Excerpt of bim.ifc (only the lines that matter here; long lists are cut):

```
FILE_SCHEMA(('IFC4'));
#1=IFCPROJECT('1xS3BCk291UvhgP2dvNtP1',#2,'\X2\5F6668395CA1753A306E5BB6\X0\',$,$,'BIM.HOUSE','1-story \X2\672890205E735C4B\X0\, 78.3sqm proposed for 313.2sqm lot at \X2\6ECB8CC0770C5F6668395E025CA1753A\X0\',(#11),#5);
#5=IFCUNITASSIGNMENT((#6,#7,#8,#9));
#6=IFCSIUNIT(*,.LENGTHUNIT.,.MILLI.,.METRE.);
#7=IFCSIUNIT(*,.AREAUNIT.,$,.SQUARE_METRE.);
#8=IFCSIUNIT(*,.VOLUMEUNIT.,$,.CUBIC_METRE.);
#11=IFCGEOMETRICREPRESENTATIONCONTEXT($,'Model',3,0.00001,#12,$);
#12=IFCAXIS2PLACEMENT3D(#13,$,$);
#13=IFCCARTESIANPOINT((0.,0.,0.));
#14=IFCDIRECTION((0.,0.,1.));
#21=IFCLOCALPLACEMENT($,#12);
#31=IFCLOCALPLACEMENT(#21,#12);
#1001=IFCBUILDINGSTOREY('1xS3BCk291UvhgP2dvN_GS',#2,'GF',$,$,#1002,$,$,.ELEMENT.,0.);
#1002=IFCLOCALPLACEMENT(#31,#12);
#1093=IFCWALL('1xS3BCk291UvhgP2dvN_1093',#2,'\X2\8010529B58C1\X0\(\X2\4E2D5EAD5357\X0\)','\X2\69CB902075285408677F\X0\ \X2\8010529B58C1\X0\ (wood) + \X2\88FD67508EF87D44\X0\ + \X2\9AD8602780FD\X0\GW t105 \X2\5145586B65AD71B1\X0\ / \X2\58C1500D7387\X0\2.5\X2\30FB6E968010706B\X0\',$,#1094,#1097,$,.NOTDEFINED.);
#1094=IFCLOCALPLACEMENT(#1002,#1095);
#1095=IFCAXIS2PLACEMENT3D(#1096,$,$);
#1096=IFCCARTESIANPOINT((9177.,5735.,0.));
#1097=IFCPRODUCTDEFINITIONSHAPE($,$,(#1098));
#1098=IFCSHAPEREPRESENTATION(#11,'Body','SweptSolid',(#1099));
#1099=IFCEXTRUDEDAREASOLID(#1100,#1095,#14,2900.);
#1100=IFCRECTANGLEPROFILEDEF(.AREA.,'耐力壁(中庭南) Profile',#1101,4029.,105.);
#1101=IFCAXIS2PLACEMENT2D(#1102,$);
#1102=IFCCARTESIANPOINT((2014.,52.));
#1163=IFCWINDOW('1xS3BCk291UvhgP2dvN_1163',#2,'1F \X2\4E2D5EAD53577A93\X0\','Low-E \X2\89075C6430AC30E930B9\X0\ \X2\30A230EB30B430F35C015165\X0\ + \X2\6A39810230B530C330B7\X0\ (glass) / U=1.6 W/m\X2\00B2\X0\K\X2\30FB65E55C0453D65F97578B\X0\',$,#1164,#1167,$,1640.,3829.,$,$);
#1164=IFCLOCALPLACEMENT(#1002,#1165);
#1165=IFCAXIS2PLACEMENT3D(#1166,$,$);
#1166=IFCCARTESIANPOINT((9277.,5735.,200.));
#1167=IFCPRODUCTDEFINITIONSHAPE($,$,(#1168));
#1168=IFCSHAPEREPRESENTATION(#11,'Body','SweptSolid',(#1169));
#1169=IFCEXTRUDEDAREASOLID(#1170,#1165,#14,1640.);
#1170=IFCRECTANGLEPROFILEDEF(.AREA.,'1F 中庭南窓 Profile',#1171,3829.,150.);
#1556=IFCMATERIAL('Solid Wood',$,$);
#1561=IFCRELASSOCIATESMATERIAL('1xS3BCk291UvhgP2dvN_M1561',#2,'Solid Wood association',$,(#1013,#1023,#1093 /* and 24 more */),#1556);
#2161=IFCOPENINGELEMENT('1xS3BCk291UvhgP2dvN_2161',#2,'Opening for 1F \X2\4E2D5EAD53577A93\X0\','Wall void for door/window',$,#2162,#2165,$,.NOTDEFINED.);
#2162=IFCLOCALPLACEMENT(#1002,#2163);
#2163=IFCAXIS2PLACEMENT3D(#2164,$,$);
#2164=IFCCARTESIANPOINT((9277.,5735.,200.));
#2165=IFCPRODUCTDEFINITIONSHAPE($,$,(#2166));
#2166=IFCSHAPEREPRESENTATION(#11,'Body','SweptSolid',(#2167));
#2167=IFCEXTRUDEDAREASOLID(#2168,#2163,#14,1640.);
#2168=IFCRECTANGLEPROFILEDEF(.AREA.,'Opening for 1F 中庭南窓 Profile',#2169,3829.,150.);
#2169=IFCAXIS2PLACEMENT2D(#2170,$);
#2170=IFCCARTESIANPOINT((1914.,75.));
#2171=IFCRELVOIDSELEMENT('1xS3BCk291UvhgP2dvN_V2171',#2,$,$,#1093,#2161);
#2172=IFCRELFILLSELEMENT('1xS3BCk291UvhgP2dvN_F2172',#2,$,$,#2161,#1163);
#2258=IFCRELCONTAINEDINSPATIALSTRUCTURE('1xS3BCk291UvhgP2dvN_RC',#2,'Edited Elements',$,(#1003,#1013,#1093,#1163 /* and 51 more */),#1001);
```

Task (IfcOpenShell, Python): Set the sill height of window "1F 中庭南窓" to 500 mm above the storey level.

```python
import numpy as np
import ifcopenshell
import ifcopenshell.api.geometry
import ifcopenshell.geom
import ifcopenshell.util.element
import ifcopenshell.util.placement
import ifcopenshell.util.shape
import ifcopenshell.util.unit

model = ifcopenshell.open("bim.ifc")
unit_scale = ifcopenshell.util.unit.calculate_unit_scale(model)

window = model.by_guid("1xS3BCk291UvhgP2dvN_1163")
opening = window.FillsVoids[0].RelatingOpeningElement
storey = ifcopenshell.util.element.get_container(window, ifc_class="IfcBuildingStorey")
level = ifcopenshell.util.placement.get_local_placement(storey.ObjectPlacement)[2, 3]

# The opening's origin need not be at the sill, so measure its lowest point.
shape = ifcopenshell.geom.create_shape(ifcopenshell.geom.settings(), opening)
bottom = ifcopenshell.util.shape.get_shape_bottom_elevation(shape, shape.geometry) / unit_scale
dz = level + 0.5 / unit_scale - bottom

shift = np.array([0.0, 0.0, dz])
# The window is not placed relative to its opening, so move both.
for product in (opening, window):
    matrix = ifcopenshell.util.placement.get_local_placement(product.ObjectPlacement)
    matrix[:3, 3] += shift
    ifcopenshell.api.geometry.edit_object_placement(model, product=product, matrix=matrix, is_si=False)

print(f"moved by {dz * unit_scale:+.3f} m")

model.write("bim_rev.ifc")
```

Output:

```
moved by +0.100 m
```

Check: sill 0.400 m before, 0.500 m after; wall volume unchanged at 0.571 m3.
